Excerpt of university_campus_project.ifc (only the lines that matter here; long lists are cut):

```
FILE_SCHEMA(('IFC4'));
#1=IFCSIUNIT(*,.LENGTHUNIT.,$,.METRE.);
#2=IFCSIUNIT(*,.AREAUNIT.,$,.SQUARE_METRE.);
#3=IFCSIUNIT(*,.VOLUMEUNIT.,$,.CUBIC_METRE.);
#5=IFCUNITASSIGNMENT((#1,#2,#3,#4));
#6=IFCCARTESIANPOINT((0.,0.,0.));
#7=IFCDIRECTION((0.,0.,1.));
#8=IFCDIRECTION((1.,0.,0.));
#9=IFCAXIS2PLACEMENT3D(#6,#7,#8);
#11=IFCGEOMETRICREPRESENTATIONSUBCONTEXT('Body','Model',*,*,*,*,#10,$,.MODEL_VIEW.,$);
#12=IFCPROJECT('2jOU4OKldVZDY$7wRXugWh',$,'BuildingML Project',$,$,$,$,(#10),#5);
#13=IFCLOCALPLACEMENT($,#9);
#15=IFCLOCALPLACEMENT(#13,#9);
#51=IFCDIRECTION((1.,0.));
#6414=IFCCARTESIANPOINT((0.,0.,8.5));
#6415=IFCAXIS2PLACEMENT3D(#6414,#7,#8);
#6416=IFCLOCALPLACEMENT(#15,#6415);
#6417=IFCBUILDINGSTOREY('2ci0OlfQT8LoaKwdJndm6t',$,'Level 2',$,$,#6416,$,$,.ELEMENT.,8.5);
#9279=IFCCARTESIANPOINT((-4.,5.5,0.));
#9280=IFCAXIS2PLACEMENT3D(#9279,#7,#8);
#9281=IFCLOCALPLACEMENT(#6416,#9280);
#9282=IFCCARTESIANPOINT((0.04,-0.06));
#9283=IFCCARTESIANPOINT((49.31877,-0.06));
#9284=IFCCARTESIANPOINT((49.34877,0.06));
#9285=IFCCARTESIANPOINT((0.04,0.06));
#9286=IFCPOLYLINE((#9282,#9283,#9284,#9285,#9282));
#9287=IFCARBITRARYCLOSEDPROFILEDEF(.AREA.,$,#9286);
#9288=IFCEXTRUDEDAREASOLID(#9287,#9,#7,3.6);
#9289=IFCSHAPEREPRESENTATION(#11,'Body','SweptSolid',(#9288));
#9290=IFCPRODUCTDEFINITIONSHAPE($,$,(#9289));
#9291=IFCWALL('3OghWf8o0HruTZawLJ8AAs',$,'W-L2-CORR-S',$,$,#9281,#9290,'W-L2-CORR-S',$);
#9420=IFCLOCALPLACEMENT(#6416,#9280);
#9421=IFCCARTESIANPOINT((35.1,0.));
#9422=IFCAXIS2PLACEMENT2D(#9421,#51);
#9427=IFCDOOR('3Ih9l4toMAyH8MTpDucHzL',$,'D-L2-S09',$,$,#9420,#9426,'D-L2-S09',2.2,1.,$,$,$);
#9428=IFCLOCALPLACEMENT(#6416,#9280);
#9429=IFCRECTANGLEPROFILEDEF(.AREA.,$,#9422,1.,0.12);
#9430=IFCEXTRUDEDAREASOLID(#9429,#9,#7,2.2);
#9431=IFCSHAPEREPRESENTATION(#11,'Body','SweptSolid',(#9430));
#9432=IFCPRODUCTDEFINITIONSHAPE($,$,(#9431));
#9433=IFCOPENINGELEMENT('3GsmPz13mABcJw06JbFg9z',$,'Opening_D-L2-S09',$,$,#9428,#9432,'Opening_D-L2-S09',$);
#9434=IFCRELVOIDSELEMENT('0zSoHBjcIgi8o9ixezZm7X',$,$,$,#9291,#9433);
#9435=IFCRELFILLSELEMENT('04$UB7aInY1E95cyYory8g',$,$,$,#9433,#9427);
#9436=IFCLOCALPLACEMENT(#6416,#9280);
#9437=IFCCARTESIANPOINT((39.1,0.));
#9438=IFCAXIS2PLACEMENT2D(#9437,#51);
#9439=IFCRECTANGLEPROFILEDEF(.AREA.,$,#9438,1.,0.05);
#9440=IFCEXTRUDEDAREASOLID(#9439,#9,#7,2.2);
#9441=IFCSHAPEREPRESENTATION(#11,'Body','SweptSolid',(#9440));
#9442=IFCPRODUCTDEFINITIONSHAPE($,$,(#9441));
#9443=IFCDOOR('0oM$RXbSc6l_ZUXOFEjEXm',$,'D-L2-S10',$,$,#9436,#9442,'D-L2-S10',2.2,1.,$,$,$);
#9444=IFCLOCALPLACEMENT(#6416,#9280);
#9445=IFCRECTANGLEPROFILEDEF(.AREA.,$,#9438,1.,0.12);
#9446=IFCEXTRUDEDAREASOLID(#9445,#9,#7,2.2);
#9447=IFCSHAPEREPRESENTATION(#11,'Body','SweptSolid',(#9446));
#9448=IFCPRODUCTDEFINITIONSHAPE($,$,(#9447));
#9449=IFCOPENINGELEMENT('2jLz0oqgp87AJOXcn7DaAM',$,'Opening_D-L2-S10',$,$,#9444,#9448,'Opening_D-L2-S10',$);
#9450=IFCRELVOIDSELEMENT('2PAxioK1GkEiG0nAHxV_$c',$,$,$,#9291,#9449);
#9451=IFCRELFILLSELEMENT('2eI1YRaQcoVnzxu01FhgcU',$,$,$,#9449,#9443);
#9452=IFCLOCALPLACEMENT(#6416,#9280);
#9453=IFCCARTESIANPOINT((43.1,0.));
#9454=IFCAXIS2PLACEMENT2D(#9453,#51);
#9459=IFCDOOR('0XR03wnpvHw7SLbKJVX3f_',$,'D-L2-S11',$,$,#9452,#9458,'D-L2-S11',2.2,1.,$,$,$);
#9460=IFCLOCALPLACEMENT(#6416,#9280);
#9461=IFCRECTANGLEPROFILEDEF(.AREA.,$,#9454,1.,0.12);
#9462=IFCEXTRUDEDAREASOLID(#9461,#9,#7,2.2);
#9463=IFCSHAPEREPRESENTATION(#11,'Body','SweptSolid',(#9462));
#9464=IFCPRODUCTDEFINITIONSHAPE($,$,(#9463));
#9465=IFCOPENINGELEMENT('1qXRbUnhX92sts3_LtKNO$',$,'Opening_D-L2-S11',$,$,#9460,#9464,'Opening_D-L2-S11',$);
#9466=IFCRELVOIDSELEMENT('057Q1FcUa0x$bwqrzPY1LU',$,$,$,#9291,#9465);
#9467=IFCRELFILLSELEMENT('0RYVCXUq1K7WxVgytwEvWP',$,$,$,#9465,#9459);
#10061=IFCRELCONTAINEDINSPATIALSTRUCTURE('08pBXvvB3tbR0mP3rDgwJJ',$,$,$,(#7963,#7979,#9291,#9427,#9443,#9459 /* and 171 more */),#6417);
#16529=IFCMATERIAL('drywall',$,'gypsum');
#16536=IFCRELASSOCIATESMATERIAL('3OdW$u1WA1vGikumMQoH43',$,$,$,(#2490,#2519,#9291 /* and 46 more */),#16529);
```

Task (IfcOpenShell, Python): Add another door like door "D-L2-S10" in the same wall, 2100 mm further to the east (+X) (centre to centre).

```python
import ifcopenshell
import ifcopenshell.api.feature
import ifcopenshell.api.geometry
import ifcopenshell.api.root
import ifcopenshell.geom
import ifcopenshell.util.element
import ifcopenshell.util.placement
import ifcopenshell.util.shape
import ifcopenshell.util.unit

model = ifcopenshell.open("university_campus_project.ifc")
unit_scale = ifcopenshell.util.unit.calculate_unit_scale(model)
settings = ifcopenshell.geom.settings()


def volume(element):
    """Net volume in cubic metres, openings subtracted."""
    shape = ifcopenshell.geom.create_shape(settings, element)
    return ifcopenshell.util.shape.get_volume(shape.geometry)


door = model.by_guid("0oM$RXbSc6l_ZUXOFEjEXm")
opening = door.FillsVoids[0].RelatingOpeningElement
wall = opening.VoidsElements[0].RelatingBuildingElement
before = volume(wall)
shift = ifcopenshell.util.placement.get_local_placement(wall.ObjectPlacement)[:3, 0] * 2.1 / unit_scale

# copy_class copies the void relationship, type, container and properties, but no geometry.
new_opening = ifcopenshell.api.root.copy_class(model, product=opening)
new_opening.Representation = ifcopenshell.util.element.copy_deep(
    model, opening.Representation, exclude=["IfcGeometricRepresentationContext", "IfcRepresentationMap"]
)
new_opening.Tag = None
new_door = ifcopenshell.api.root.copy_class(model, product=door)
new_door.Representation = ifcopenshell.util.element.copy_deep(
    model, door.Representation, exclude=["IfcGeometricRepresentationContext", "IfcRepresentationMap"]
)
new_door.Tag = None
ifcopenshell.api.feature.add_filling(model, opening=new_opening, element=new_door)

for old, new in ((opening, new_opening), (door, new_door)):
    matrix = ifcopenshell.util.placement.get_local_placement(old.ObjectPlacement)
    matrix[:3, 3] += shift
    ifcopenshell.api.geometry.edit_object_placement(model, product=new, matrix=matrix, is_si=False)

after = volume(wall)

print(f"wall volume {before:.3f} -> {after:.3f} m3")

model.write("university_campus_project_edited.ifc")
```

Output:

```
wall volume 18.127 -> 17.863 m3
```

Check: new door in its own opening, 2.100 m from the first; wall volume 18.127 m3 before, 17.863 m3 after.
